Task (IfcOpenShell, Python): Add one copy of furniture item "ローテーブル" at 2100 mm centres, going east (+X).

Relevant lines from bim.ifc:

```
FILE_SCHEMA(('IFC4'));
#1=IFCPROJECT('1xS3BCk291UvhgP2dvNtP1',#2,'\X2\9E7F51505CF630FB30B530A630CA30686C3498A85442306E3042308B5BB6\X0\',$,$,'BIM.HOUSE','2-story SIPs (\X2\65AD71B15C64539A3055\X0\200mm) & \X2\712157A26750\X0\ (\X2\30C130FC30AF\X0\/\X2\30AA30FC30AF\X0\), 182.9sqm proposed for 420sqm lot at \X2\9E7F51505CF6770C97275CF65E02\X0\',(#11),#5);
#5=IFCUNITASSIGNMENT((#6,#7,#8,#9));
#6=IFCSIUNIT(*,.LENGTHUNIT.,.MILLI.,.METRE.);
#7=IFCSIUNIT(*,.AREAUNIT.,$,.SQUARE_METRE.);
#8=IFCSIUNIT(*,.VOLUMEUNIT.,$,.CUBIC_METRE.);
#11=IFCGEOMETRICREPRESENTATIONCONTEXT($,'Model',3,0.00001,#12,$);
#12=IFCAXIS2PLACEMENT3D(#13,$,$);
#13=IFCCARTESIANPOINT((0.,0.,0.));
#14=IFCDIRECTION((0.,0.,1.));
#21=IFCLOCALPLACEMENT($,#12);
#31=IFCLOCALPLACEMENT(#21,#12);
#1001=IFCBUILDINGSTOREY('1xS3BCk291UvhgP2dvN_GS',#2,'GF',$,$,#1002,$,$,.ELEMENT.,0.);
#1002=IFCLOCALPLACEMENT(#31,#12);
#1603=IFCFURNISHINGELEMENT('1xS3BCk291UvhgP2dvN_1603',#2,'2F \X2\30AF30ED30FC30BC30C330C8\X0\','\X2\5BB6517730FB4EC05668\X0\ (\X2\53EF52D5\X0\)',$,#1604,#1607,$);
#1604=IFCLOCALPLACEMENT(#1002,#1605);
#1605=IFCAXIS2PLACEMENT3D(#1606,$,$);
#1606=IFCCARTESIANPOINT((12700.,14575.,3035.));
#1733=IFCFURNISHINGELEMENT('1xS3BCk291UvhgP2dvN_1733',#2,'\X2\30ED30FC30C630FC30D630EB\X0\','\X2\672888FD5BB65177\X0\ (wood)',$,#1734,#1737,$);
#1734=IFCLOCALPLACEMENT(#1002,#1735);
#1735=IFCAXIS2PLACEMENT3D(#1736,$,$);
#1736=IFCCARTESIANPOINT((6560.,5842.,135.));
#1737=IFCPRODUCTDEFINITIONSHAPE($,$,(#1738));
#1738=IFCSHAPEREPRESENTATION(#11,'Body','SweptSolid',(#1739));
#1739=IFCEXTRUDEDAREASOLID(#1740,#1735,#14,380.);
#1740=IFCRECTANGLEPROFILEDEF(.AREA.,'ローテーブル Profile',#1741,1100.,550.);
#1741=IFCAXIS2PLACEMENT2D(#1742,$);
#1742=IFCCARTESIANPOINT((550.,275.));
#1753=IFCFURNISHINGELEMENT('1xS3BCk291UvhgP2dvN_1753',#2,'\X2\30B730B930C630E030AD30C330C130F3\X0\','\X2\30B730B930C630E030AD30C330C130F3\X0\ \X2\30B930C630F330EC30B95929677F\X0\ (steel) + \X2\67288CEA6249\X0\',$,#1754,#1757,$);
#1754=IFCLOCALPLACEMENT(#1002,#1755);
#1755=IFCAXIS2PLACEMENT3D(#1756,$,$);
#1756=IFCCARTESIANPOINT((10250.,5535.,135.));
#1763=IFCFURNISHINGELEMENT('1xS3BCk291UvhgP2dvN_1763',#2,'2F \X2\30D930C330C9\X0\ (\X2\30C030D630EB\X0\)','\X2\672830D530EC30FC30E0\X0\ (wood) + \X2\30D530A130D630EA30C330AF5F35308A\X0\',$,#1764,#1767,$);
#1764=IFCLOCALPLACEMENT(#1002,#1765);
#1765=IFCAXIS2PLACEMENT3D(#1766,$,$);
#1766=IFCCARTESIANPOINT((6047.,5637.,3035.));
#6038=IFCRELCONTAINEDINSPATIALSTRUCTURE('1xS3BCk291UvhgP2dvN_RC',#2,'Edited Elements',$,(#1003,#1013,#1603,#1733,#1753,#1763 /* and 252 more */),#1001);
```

```python
import numpy as np
import ifcopenshell
import ifcopenshell.api.geometry
import ifcopenshell.api.root
import ifcopenshell.util.element
import ifcopenshell.util.placement

model = ifcopenshell.open("bim.ifc")


def reuse_history(source, copy):
    """copy_class also copies each property set's owner history, people and application; keep the originals."""
    for rel in copy.IsDefinedBy:
        if rel.is_a("IfcRelDefinesByProperties") and (history := rel.RelatingPropertyDefinition.OwnerHistory):
            rel.RelatingPropertyDefinition.OwnerHistory = source.OwnerHistory
            ifcopenshell.util.element.remove_deep2(model, history)


source = model.by_guid("1xS3BCk291UvhgP2dvN_1733")
base = ifcopenshell.util.placement.get_local_placement(source.ObjectPlacement)
step = np.array([1.0, 0.0, 0.0]) * 2100.0

for i in range(1, 2):
    copy = ifcopenshell.api.root.copy_class(model, product=source)
    copy.Representation = ifcopenshell.util.element.copy_deep(
        model, source.Representation, exclude=["IfcGeometricRepresentationContext", "IfcRepresentationMap"]
    )
    reuse_history(source, copy)
    matrix = base.copy()
    matrix[:3, 3] += i * step
    print("added at", matrix[:3, 3].round(3) + 0.0)
    ifcopenshell.api.geometry.edit_object_placement(model, product=copy, matrix=matrix, is_si=False)

model.write("bim_edited.ifc")
```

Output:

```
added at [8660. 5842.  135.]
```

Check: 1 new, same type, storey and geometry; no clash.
